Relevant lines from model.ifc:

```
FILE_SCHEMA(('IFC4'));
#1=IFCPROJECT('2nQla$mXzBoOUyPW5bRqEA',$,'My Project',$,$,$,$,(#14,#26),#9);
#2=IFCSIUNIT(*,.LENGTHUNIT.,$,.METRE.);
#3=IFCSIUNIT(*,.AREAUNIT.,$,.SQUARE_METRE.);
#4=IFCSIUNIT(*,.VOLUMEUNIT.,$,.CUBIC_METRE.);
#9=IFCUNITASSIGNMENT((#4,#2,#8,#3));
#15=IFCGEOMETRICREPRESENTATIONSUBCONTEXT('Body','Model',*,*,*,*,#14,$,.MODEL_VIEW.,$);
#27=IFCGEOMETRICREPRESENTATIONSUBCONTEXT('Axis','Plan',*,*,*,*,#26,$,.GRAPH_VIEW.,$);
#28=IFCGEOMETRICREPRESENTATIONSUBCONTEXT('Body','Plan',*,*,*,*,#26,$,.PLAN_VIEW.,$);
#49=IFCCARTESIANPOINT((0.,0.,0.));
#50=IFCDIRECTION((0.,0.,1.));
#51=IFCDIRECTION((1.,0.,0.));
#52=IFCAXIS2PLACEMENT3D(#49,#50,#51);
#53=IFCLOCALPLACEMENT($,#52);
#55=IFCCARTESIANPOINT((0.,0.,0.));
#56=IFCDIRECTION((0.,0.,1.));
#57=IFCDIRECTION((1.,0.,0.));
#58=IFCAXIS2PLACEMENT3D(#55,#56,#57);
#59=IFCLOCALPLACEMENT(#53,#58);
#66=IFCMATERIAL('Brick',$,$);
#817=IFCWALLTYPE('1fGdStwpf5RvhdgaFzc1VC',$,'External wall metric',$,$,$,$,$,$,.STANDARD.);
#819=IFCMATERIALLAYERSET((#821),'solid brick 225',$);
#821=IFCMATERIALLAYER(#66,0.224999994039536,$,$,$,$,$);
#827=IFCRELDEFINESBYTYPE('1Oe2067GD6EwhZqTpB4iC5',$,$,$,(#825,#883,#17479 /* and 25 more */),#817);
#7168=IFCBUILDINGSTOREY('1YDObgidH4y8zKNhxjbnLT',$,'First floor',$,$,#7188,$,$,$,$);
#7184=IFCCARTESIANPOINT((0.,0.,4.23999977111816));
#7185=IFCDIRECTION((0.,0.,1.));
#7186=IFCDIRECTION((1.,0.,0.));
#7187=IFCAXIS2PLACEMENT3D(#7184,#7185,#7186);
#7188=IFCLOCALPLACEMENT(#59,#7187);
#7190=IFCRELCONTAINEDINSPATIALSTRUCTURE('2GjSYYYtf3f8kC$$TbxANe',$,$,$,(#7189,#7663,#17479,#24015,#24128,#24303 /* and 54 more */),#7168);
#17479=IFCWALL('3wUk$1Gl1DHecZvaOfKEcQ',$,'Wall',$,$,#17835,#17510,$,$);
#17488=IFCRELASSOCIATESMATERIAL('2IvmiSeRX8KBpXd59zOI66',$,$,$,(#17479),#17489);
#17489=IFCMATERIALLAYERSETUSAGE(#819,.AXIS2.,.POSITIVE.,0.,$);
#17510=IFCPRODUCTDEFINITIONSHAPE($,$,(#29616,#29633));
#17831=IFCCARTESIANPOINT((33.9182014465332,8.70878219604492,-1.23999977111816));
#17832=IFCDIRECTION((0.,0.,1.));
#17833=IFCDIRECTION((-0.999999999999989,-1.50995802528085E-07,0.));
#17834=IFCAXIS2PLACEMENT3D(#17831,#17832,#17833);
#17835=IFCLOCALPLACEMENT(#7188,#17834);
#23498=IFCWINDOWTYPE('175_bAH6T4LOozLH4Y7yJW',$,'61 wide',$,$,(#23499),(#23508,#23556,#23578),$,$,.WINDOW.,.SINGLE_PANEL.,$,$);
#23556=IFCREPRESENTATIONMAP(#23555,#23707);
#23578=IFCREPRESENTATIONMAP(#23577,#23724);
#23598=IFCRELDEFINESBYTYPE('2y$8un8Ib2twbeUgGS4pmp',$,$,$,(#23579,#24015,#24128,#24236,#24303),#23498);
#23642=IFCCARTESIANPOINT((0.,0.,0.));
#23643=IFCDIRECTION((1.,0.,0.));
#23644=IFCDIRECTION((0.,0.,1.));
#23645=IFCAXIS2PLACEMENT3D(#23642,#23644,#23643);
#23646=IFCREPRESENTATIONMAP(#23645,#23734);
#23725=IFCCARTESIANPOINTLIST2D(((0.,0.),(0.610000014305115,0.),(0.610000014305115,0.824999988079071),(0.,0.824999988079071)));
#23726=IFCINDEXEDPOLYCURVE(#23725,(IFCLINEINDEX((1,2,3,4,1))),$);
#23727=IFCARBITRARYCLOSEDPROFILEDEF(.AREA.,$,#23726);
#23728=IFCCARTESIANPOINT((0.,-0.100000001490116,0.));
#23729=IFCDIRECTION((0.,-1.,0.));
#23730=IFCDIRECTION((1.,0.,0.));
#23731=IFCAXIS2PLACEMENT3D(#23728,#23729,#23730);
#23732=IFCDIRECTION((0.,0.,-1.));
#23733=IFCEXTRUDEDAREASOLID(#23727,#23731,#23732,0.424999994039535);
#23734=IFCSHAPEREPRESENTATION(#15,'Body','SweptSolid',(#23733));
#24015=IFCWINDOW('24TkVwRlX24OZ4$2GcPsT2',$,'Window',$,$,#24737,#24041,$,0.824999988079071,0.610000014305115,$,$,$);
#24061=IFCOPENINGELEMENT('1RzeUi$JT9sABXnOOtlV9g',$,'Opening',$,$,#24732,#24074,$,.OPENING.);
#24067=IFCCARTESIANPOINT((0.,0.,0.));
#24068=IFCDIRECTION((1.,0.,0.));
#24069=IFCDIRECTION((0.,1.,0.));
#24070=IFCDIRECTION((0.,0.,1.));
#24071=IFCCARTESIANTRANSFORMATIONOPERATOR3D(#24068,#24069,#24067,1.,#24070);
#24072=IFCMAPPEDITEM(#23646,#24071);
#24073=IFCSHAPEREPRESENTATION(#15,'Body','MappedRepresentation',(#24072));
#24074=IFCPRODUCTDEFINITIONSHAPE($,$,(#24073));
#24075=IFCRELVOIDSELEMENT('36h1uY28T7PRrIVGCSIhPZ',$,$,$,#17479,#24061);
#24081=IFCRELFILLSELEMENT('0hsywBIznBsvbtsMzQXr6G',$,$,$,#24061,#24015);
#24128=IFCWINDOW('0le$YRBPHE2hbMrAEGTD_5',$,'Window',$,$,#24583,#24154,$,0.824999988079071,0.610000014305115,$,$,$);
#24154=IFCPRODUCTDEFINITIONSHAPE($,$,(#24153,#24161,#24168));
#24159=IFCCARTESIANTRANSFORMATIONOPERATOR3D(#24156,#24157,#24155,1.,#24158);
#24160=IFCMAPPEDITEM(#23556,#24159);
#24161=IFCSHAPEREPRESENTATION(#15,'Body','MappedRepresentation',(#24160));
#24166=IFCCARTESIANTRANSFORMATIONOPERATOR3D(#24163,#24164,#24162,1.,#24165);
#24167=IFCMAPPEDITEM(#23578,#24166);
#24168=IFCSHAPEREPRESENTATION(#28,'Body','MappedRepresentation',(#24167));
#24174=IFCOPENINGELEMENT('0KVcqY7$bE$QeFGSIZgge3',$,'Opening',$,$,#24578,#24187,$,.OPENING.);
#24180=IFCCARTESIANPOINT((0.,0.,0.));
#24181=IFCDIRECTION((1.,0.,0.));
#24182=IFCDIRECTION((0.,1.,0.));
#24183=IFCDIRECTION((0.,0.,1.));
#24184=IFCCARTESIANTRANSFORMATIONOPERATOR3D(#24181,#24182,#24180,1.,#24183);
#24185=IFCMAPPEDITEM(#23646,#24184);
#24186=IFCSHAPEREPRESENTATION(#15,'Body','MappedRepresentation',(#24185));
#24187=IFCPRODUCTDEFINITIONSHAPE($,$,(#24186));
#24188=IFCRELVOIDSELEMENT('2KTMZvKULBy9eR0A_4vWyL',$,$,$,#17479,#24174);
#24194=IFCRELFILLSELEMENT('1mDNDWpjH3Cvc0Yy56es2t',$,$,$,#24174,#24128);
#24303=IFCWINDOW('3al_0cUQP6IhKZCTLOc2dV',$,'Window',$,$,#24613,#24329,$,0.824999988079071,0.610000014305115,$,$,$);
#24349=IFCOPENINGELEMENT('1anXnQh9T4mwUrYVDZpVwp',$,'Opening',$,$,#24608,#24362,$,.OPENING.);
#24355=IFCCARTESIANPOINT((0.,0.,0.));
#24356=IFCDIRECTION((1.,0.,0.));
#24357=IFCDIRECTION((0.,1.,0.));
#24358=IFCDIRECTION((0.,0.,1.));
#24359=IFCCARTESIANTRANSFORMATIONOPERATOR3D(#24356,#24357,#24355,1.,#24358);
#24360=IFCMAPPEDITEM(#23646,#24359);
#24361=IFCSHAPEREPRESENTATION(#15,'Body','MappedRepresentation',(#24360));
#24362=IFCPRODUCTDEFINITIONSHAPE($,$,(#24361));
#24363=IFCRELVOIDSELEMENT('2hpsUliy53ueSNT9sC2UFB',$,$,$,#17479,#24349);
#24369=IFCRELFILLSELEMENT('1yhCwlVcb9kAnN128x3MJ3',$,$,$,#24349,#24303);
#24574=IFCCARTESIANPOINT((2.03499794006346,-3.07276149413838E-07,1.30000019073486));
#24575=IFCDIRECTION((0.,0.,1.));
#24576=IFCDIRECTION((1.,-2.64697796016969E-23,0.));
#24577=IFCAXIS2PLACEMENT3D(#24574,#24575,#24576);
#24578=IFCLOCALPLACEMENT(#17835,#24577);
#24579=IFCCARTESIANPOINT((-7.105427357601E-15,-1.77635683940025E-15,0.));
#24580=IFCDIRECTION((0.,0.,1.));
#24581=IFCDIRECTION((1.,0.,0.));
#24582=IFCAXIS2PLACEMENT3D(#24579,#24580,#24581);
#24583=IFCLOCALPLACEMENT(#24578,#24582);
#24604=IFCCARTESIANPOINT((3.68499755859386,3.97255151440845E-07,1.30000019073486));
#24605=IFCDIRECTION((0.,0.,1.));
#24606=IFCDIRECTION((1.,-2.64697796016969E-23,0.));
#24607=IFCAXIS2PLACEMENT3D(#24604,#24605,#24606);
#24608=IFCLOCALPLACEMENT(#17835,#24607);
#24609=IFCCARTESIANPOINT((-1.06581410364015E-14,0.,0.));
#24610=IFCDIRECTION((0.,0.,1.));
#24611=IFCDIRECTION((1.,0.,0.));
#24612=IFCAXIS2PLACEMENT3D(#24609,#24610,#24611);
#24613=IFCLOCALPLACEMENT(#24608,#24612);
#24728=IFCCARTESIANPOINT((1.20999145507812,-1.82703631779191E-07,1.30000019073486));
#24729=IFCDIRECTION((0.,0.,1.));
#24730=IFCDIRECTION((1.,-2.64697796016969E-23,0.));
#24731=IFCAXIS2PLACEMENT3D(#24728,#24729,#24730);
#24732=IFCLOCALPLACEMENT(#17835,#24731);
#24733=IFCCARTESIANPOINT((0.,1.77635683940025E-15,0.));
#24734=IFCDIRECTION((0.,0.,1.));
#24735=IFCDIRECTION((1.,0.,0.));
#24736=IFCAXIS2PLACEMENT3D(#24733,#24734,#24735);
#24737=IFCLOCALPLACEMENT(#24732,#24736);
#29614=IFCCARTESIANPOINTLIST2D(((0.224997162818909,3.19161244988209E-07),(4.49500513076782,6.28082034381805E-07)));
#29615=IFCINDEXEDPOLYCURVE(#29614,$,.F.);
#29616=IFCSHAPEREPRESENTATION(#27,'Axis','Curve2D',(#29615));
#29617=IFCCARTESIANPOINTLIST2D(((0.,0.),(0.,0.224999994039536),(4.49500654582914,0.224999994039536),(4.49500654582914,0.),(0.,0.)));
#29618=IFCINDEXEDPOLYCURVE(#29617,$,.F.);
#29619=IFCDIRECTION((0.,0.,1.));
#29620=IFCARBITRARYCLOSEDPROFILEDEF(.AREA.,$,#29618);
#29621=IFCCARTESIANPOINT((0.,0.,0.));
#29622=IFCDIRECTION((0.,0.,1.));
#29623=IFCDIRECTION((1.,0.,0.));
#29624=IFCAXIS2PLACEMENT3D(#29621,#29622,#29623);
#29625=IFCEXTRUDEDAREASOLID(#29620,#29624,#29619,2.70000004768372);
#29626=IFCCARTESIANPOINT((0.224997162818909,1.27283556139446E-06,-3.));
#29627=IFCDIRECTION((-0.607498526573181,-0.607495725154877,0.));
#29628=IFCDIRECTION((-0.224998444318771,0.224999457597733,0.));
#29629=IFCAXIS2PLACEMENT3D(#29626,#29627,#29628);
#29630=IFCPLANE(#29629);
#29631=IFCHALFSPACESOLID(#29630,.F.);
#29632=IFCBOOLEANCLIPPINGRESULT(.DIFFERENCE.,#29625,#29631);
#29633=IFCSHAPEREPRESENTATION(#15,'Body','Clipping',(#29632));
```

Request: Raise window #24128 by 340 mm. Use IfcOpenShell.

```python
import numpy as np
import ifcopenshell
import ifcopenshell.api.geometry
import ifcopenshell.util.placement
import ifcopenshell.util.unit

model = ifcopenshell.open("model.ifc")
unit_scale = ifcopenshell.util.unit.calculate_unit_scale(model)

window = model.by_guid("0le$YRBPHE2hbMrAEGTD_5")
opening = window.FillsVoids[0].RelatingOpeningElement
dz = 0.34

shift = np.array([0.0, 0.0, dz])
# The window is placed relative to its opening, so it follows when the opening moves.
matrix = ifcopenshell.util.placement.get_local_placement(opening.ObjectPlacement)
matrix[:3, 3] += shift
ifcopenshell.api.geometry.edit_object_placement(
    model, product=opening, matrix=matrix, is_si=False, should_transform_children=True
)

print(f"moved by {dz * unit_scale:+.3f} m")

model.write("model_v2.ifc")
```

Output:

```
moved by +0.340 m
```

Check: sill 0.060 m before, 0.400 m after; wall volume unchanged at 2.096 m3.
